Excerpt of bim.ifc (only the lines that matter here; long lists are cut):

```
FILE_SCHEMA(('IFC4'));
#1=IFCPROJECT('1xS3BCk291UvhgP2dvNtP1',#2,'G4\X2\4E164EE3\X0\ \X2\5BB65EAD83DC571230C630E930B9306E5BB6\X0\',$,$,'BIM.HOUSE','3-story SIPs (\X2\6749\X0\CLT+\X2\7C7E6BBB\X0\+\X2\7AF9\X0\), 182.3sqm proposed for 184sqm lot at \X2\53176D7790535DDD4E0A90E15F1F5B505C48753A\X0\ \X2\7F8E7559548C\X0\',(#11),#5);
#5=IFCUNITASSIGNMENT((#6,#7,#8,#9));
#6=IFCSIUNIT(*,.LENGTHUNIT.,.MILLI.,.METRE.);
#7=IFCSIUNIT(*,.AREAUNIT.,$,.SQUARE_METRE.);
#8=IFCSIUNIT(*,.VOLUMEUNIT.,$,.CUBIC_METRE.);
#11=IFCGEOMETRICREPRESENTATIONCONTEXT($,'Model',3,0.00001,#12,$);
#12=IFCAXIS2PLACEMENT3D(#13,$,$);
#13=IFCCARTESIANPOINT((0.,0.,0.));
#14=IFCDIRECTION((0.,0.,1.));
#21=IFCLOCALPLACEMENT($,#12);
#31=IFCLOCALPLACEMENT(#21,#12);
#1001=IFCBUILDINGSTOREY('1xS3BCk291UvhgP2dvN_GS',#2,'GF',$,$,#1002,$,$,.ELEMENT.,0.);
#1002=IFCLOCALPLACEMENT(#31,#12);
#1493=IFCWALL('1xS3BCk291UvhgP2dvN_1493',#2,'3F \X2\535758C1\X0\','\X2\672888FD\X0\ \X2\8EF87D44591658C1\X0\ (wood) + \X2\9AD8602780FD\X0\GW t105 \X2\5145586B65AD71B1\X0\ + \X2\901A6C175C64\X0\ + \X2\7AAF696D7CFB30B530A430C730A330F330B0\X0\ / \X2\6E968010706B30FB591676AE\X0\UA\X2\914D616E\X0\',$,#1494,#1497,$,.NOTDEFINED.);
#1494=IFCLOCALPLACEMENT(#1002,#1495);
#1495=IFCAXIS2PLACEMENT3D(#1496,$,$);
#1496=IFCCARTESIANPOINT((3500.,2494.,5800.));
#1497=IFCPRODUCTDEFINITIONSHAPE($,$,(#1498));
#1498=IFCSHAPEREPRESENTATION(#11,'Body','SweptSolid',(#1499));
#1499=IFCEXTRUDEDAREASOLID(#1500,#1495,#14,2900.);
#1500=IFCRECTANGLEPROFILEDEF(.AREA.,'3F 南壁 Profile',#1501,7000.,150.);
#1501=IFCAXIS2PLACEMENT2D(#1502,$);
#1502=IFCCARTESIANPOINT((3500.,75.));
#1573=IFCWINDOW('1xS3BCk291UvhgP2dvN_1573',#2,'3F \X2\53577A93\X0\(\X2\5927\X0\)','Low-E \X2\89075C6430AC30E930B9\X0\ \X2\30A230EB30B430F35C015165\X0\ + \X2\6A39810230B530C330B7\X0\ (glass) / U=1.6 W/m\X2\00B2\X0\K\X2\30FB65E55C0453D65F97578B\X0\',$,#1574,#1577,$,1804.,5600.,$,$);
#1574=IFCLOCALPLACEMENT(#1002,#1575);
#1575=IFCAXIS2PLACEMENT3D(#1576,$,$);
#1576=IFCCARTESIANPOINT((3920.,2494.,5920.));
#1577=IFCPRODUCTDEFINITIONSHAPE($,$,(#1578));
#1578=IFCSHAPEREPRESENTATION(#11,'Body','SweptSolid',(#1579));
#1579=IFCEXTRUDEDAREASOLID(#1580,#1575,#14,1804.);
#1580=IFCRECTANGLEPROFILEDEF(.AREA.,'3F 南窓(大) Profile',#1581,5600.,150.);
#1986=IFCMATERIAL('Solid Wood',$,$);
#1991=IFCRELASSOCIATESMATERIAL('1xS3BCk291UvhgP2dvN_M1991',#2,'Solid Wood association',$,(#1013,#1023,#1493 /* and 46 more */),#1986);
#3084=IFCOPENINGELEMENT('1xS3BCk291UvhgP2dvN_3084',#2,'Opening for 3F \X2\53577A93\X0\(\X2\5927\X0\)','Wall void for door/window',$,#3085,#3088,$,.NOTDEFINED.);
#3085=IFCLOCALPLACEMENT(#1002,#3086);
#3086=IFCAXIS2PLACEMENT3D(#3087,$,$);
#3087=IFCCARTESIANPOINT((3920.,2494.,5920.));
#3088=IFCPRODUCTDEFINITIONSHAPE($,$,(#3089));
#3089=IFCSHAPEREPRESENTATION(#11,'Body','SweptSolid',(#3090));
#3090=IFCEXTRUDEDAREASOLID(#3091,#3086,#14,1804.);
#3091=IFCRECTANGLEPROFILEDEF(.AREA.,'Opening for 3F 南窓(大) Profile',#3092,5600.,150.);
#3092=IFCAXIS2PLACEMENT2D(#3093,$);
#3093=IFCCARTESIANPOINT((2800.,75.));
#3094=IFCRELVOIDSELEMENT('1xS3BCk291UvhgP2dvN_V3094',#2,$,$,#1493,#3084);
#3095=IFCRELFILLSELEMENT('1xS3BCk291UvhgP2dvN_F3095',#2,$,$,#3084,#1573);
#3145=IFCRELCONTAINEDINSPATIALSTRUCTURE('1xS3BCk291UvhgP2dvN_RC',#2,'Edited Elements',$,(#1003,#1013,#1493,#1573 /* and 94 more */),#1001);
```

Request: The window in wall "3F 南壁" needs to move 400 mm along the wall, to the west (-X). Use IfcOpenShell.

```python
import ifcopenshell
import ifcopenshell.api.geometry
import ifcopenshell.util.placement
import ifcopenshell.util.unit

model = ifcopenshell.open("bim.ifc")
unit_scale = ifcopenshell.util.unit.calculate_unit_scale(model)

window = model.by_guid("1xS3BCk291UvhgP2dvN_1573")
opening = window.FillsVoids[0].RelatingOpeningElement
wall = opening.VoidsElements[0].RelatingBuildingElement

wall_matrix = ifcopenshell.util.placement.get_local_placement(wall.ObjectPlacement)
shift = wall_matrix[:3, 0] * -0.4 / unit_scale
before = ifcopenshell.util.placement.get_local_placement(window.ObjectPlacement)[:3, 3].copy()

# The window is not placed relative to its opening, so move both.
for product in (opening, window):
    matrix = ifcopenshell.util.placement.get_local_placement(product.ObjectPlacement)
    matrix[:3, 3] += shift
    ifcopenshell.api.geometry.edit_object_placement(model, product=product, matrix=matrix, is_si=False)

after = ifcopenshell.util.placement.get_local_placement(window.ObjectPlacement)[:3, 3]
print("window moved by", (after - before).round(3) + 0.0)

model.write("bim_v2.ifc")
```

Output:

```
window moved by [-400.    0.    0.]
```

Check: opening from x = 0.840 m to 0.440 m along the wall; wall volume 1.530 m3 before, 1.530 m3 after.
